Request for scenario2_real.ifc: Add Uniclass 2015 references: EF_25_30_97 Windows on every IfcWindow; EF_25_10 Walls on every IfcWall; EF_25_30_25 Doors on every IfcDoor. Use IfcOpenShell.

First a look at what the model holds.

```python
import ifcopenshell

model = ifcopenshell.open("scenario2_real.ifc")
print(model.schema)
print("classifications:", [c.Name for c in model.by_type("IfcClassification")])
for ifc_class in ("IfcDoor", "IfcRoof", "IfcStair", "IfcWall", "IfcWindow"):
    print(ifc_class, len(model.by_type(ifc_class)))
```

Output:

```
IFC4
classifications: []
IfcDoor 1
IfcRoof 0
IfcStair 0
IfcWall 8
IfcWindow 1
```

```python
import ifcopenshell
import ifcopenshell.api.classification

model = ifcopenshell.open("scenario2_real.ifc")

system = ifcopenshell.api.classification.add_classification(model, classification="Uniclass 2015")

codes = {
    "IfcWindow": ("EF_25_30_97", "Windows"),
    "IfcWall": ("EF_25_10", "Walls"),
    "IfcDoor": ("EF_25_30_25", "Doors"),
}
for ifc_class, (code, name) in codes.items():
    products = model.by_type(ifc_class)
    ifcopenshell.api.classification.add_reference(
        model, products=products, classification=system, identification=code, name=name
    )
    print(code, len(products))

model.write("scenario2_real_v2.ifc")
```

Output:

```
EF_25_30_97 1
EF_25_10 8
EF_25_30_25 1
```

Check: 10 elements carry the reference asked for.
